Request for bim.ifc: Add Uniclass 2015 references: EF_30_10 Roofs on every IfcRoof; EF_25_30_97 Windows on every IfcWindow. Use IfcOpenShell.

First a look at what the model holds.

```python
import ifcopenshell

model = ifcopenshell.open("bim.ifc")
print(model.schema)
print("classifications:", [c.Name for c in model.by_type("IfcClassification")])
for ifc_class in ("IfcDoor", "IfcRoof", "IfcStair", "IfcWall", "IfcWindow"):
    print(ifc_class, len(model.by_type(ifc_class)))
```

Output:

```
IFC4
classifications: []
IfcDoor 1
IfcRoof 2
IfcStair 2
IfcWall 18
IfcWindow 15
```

```python
import ifcopenshell
import ifcopenshell.api.classification

model = ifcopenshell.open("bim.ifc")

system = ifcopenshell.api.classification.add_classification(model, classification="Uniclass 2015")

codes = {
    "IfcRoof": ("EF_30_10", "Roofs"),
    "IfcWindow": ("EF_25_30_97", "Windows"),
}
for ifc_class, (code, name) in codes.items():
    products = model.by_type(ifc_class)
    ifcopenshell.api.classification.add_reference(
        model, products=products, classification=system, identification=code, name=name
    )
    print(code, len(products))

model.write("bim_edited.ifc")
```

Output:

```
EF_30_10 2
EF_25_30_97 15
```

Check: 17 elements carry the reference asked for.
